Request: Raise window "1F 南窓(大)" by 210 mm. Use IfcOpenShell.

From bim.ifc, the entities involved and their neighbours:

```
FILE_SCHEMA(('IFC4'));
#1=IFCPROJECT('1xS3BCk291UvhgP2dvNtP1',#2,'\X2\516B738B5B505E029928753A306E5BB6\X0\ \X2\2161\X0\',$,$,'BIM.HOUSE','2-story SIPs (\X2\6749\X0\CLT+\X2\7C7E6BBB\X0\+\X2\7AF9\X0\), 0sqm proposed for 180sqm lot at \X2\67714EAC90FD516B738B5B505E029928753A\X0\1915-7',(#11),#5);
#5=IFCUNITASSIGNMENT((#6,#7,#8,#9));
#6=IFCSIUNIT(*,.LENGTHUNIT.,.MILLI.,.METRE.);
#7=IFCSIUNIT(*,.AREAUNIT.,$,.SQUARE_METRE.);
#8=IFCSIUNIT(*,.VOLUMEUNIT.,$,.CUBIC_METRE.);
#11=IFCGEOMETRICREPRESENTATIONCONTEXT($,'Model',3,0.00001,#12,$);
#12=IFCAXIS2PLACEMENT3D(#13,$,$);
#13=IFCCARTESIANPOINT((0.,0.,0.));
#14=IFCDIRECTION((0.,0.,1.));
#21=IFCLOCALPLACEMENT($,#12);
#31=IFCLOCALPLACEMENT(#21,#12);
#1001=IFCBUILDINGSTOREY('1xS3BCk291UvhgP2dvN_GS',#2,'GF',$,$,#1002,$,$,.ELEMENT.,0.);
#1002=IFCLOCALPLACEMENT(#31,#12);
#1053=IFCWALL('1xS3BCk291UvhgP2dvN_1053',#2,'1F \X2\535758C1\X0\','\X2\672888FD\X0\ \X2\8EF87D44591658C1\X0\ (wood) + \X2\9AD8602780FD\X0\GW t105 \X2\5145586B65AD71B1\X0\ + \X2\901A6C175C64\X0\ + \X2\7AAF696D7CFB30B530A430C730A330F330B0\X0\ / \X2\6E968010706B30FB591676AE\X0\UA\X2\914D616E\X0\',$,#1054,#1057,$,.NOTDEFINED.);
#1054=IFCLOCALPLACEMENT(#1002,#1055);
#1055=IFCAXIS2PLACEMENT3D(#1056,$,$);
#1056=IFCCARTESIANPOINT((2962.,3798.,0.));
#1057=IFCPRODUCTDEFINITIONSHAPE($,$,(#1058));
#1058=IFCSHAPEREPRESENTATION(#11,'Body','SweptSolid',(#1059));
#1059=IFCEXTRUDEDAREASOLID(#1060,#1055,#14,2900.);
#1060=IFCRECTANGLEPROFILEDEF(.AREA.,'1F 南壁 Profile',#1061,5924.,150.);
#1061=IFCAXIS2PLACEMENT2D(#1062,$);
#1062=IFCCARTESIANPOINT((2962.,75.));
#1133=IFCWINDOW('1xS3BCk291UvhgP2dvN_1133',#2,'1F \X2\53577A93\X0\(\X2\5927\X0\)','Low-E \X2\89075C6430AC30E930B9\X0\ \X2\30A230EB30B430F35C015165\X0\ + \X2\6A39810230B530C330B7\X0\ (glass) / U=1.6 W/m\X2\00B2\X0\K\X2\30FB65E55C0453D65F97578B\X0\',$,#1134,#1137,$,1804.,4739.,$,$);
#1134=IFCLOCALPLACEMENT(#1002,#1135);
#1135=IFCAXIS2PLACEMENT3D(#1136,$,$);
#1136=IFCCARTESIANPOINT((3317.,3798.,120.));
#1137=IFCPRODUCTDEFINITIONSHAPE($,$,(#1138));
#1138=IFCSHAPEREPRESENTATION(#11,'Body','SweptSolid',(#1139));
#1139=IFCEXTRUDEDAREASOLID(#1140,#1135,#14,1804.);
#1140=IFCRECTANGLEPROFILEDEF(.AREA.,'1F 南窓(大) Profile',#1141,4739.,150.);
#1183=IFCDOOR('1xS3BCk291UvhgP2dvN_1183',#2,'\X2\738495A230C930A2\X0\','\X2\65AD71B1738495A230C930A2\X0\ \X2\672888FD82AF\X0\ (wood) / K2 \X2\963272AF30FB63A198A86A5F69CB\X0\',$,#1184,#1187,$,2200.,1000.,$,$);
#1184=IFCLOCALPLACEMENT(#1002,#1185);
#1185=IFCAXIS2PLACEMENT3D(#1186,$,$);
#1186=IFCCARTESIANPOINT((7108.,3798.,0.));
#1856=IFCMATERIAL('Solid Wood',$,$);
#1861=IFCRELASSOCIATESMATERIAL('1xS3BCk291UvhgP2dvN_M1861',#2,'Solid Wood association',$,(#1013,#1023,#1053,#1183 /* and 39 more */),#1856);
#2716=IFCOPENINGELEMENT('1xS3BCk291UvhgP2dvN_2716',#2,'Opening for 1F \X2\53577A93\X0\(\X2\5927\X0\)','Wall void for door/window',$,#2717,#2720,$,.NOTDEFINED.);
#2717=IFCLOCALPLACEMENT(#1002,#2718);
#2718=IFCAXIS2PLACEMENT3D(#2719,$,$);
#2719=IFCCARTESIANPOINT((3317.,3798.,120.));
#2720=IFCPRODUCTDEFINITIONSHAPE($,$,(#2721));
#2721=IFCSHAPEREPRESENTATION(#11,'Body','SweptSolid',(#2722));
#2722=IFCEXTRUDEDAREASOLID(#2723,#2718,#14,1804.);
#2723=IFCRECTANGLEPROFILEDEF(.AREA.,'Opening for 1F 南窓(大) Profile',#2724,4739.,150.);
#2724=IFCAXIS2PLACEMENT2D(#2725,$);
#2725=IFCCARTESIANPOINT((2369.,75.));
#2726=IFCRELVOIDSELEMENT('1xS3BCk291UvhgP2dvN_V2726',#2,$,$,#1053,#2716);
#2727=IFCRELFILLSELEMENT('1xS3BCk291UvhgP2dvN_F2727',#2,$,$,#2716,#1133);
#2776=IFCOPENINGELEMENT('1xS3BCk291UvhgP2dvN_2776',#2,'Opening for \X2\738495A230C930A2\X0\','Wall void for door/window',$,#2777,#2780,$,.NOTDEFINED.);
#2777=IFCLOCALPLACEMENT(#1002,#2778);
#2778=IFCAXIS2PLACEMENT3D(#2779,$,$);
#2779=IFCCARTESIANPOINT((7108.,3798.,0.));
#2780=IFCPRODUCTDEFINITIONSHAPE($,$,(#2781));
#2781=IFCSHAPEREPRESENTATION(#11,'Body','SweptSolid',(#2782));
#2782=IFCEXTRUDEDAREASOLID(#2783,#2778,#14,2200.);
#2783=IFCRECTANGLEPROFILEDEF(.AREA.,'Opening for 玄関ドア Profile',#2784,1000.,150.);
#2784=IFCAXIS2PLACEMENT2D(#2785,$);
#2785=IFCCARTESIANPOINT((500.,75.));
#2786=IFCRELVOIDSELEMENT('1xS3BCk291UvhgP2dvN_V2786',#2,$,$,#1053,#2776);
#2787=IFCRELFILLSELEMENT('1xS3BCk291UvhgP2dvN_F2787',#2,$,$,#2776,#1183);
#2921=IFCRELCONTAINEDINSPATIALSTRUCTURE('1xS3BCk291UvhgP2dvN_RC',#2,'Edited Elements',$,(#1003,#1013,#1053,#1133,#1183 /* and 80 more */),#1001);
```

```python
import numpy as np
import ifcopenshell
import ifcopenshell.api.geometry
import ifcopenshell.util.placement
import ifcopenshell.util.unit

model = ifcopenshell.open("bim.ifc")
unit_scale = ifcopenshell.util.unit.calculate_unit_scale(model)

window = model.by_guid("1xS3BCk291UvhgP2dvN_1133")
opening = window.FillsVoids[0].RelatingOpeningElement
dz = 210.0

shift = np.array([0.0, 0.0, dz])
# The window is not placed relative to its opening, so move both.
for product in (opening, window):
    matrix = ifcopenshell.util.placement.get_local_placement(product.ObjectPlacement)
    matrix[:3, 3] += shift
    ifcopenshell.api.geometry.edit_object_placement(model, product=product, matrix=matrix, is_si=False)

print(f"moved by {dz * unit_scale:+.3f} m")

model.write("bim_edited.ifc")
```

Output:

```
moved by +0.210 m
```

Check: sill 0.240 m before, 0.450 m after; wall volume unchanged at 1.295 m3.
